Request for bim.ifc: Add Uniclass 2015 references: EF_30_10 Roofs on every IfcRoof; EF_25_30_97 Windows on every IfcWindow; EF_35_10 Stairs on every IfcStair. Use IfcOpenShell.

First a look at what the model holds.

```python
import ifcopenshell

model = ifcopenshell.open("bim.ifc")
print(model.schema)
print("classifications:", [c.Name for c in model.by_type("IfcClassification")])
for ifc_class in ("IfcDoor", "IfcRoof", "IfcStair", "IfcWall", "IfcWindow"):
    print(ifc_class, len(model.by_type(ifc_class)))
```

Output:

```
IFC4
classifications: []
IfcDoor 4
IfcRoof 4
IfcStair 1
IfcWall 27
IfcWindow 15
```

```python
import ifcopenshell
import ifcopenshell.api.classification

model = ifcopenshell.open("bim.ifc")

system = ifcopenshell.api.classification.add_classification(model, classification="Uniclass 2015")

codes = {
    "IfcRoof": ("EF_30_10", "Roofs"),
    "IfcWindow": ("EF_25_30_97", "Windows"),
    "IfcStair": ("EF_35_10", "Stairs"),
}
for ifc_class, (code, name) in codes.items():
    products = model.by_type(ifc_class)
    ifcopenshell.api.classification.add_reference(
        model, products=products, classification=system, identification=code, name=name
    )
    print(code, len(products))

model.write("bim_updated.ifc")
```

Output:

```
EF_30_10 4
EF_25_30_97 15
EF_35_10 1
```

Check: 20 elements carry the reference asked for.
